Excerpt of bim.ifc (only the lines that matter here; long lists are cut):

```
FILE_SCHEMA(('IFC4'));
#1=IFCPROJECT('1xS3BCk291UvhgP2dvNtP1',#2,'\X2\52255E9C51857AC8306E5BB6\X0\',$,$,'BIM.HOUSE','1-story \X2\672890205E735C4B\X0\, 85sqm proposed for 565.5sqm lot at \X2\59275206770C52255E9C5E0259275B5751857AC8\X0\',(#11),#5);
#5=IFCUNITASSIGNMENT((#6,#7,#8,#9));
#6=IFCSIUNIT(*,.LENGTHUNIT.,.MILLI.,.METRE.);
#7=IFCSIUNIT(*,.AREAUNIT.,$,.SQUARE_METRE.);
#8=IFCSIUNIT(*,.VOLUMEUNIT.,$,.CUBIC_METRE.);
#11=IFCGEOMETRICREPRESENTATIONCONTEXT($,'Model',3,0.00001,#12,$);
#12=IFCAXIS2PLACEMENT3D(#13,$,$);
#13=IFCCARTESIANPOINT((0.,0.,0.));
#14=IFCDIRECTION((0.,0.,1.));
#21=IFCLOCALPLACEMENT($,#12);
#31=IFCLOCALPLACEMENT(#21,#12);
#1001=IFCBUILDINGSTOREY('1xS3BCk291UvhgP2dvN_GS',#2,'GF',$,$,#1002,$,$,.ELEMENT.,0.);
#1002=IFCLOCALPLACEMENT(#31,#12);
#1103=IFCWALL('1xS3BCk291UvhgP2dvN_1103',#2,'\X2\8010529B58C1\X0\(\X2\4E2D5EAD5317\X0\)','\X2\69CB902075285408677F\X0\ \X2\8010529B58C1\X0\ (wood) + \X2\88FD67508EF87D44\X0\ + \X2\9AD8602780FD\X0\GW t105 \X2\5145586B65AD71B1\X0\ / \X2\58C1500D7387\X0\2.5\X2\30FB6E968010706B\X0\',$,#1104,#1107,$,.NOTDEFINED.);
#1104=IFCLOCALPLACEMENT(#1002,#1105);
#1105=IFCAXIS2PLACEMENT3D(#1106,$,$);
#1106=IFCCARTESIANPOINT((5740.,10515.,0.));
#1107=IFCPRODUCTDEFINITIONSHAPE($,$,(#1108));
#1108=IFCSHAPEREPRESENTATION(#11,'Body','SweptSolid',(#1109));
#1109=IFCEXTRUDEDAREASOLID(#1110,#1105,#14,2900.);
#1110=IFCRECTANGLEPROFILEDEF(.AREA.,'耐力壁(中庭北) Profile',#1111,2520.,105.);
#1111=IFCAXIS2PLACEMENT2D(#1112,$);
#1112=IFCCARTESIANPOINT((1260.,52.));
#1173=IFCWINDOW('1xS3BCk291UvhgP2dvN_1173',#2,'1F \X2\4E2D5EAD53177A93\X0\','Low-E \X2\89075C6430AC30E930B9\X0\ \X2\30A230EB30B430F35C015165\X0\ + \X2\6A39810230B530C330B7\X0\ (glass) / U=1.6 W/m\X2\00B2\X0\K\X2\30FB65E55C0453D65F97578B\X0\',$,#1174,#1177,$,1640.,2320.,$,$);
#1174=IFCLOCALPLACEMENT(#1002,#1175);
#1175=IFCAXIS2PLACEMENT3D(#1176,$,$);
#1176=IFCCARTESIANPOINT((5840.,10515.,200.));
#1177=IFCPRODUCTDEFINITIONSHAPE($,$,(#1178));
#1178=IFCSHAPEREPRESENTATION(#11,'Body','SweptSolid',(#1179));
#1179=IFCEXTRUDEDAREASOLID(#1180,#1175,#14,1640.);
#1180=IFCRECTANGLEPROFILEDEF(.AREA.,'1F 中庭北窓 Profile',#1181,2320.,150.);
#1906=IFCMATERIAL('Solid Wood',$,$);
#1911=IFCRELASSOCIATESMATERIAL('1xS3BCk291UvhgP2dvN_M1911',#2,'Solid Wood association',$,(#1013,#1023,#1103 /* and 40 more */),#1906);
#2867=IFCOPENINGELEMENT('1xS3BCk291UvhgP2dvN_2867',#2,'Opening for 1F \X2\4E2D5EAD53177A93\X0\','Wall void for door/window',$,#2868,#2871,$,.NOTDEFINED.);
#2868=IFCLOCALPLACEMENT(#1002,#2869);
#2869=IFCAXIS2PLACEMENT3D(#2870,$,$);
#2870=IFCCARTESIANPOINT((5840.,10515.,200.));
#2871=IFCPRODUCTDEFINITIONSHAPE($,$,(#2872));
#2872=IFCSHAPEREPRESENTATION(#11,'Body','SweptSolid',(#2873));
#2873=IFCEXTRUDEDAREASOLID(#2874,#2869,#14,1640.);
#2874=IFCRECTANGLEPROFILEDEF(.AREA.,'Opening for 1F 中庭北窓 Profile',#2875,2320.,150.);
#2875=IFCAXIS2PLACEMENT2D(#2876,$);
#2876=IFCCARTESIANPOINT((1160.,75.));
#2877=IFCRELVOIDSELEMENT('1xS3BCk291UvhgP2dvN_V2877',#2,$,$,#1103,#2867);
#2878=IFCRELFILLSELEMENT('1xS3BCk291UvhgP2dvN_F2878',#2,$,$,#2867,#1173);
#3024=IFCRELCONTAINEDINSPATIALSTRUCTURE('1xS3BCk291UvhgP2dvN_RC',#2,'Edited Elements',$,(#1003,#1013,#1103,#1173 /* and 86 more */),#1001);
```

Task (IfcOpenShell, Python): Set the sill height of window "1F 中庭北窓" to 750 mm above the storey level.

```python
import numpy as np
import ifcopenshell
import ifcopenshell.api.geometry
import ifcopenshell.geom
import ifcopenshell.util.element
import ifcopenshell.util.placement
import ifcopenshell.util.shape
import ifcopenshell.util.unit

model = ifcopenshell.open("bim.ifc")
unit_scale = ifcopenshell.util.unit.calculate_unit_scale(model)

window = model.by_id(1173)
opening = window.FillsVoids[0].RelatingOpeningElement
storey = ifcopenshell.util.element.get_container(window, ifc_class="IfcBuildingStorey")
level = ifcopenshell.util.placement.get_local_placement(storey.ObjectPlacement)[2, 3]

# The opening's origin need not be at the sill, so measure its lowest point.
shape = ifcopenshell.geom.create_shape(ifcopenshell.geom.settings(), opening)
bottom = ifcopenshell.util.shape.get_shape_bottom_elevation(shape, shape.geometry) / unit_scale
dz = level + 750.0 - bottom

shift = np.array([0.0, 0.0, dz])
# The window is not placed relative to its opening, so move both.
for product in (opening, window):
    matrix = ifcopenshell.util.placement.get_local_placement(product.ObjectPlacement)
    matrix[:3, 3] += shift
    ifcopenshell.api.geometry.edit_object_placement(model, product=product, matrix=matrix, is_si=False)

print(f"moved by {dz * unit_scale:+.3f} m")

model.write("bim_rev.ifc")
```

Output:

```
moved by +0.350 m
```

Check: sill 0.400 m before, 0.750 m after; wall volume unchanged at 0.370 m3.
